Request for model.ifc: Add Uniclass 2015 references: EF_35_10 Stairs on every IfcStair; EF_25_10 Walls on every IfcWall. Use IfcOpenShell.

First a look at what the model holds.

```python
import ifcopenshell

model = ifcopenshell.open("model.ifc")
print(model.schema)
print("classifications:", [c.Name for c in model.by_type("IfcClassification")])
for ifc_class in ("IfcDoor", "IfcRoof", "IfcStair", "IfcWall", "IfcWindow"):
    print(ifc_class, len(model.by_type(ifc_class)))
```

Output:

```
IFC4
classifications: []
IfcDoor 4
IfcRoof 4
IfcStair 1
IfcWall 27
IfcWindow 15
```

```python
import ifcopenshell
import ifcopenshell.api.classification

model = ifcopenshell.open("model.ifc")

system = ifcopenshell.api.classification.add_classification(model, classification="Uniclass 2015")

codes = {
    "IfcStair": ("EF_35_10", "Stairs"),
    "IfcWall": ("EF_25_10", "Walls"),
}
for ifc_class, (code, name) in codes.items():
    products = model.by_type(ifc_class)
    ifcopenshell.api.classification.add_reference(
        model, products=products, classification=system, identification=code, name=name
    )
    print(code, len(products))

model.write("model_edited.ifc")
```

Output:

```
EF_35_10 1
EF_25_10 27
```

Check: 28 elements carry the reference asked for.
